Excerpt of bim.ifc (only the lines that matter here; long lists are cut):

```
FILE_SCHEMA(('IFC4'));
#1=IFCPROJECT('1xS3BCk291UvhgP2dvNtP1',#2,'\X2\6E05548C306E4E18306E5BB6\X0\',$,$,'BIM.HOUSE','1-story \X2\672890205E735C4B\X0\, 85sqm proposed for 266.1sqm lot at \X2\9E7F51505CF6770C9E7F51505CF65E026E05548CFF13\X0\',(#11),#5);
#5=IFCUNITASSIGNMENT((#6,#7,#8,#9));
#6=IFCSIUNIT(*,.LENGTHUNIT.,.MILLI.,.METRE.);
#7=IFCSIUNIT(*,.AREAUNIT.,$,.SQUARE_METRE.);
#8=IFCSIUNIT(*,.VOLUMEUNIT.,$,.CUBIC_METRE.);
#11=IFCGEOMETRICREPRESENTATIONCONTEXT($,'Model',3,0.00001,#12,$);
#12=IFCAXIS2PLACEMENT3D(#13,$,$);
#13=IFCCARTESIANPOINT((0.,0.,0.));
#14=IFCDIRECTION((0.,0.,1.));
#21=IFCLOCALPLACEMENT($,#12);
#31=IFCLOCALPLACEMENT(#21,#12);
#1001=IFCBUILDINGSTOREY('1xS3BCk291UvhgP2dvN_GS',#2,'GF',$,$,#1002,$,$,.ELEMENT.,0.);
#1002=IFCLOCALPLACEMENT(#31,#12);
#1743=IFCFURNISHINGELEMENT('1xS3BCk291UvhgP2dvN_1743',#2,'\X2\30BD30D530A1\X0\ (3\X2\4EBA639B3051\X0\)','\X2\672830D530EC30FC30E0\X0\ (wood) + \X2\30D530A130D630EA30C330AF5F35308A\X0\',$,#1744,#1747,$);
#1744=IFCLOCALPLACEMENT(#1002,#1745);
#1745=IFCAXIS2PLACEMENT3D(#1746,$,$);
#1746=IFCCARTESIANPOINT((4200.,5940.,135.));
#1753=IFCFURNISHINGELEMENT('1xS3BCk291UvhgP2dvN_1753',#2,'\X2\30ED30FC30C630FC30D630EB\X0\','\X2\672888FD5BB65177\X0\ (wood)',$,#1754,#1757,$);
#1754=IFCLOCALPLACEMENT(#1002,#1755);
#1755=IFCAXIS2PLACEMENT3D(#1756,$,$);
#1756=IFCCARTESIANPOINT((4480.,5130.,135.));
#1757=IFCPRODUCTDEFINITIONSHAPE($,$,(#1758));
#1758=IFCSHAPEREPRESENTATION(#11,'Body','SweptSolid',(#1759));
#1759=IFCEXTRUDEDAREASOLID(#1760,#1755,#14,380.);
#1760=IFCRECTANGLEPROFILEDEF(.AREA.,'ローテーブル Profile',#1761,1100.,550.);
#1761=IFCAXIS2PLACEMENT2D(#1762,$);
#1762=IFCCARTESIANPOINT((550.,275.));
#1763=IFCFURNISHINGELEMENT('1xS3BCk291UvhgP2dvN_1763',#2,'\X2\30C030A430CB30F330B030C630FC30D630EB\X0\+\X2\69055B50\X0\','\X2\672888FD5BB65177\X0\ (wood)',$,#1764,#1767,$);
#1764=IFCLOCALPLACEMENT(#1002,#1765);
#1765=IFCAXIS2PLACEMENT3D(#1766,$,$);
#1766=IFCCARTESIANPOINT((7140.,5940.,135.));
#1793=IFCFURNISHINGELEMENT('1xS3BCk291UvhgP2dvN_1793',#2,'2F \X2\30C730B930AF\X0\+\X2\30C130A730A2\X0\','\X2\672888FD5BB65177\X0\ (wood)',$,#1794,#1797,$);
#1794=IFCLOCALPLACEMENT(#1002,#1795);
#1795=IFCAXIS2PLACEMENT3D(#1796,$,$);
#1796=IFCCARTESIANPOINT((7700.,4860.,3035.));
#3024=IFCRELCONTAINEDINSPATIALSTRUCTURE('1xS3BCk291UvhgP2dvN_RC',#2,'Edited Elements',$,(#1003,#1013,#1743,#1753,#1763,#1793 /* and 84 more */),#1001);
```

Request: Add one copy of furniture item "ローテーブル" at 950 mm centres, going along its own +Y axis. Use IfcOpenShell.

```python
import ifcopenshell
import ifcopenshell.api.geometry
import ifcopenshell.api.root
import ifcopenshell.util.element
import ifcopenshell.util.placement

model = ifcopenshell.open("bim.ifc")


def reuse_history(source, copy):
    """copy_class also copies each property set's owner history, people and application; keep the originals."""
    for rel in copy.IsDefinedBy:
        if rel.is_a("IfcRelDefinesByProperties") and (history := rel.RelatingPropertyDefinition.OwnerHistory):
            rel.RelatingPropertyDefinition.OwnerHistory = source.OwnerHistory
            ifcopenshell.util.element.remove_deep2(model, history)


source = model.by_guid("1xS3BCk291UvhgP2dvN_1753")
base = ifcopenshell.util.placement.get_local_placement(source.ObjectPlacement)
step = base[:3, 1] * 950.0

for i in range(1, 2):
    copy = ifcopenshell.api.root.copy_class(model, product=source)
    copy.Representation = ifcopenshell.util.element.copy_deep(
        model, source.Representation, exclude=["IfcGeometricRepresentationContext", "IfcRepresentationMap"]
    )
    reuse_history(source, copy)
    matrix = base.copy()
    matrix[:3, 3] += i * step
    print("added at", matrix[:3, 3].round(3) + 0.0)
    ifcopenshell.api.geometry.edit_object_placement(model, product=copy, matrix=matrix, is_si=False)

model.write("bim_edited.ifc")
```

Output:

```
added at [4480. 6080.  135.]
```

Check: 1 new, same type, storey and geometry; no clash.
